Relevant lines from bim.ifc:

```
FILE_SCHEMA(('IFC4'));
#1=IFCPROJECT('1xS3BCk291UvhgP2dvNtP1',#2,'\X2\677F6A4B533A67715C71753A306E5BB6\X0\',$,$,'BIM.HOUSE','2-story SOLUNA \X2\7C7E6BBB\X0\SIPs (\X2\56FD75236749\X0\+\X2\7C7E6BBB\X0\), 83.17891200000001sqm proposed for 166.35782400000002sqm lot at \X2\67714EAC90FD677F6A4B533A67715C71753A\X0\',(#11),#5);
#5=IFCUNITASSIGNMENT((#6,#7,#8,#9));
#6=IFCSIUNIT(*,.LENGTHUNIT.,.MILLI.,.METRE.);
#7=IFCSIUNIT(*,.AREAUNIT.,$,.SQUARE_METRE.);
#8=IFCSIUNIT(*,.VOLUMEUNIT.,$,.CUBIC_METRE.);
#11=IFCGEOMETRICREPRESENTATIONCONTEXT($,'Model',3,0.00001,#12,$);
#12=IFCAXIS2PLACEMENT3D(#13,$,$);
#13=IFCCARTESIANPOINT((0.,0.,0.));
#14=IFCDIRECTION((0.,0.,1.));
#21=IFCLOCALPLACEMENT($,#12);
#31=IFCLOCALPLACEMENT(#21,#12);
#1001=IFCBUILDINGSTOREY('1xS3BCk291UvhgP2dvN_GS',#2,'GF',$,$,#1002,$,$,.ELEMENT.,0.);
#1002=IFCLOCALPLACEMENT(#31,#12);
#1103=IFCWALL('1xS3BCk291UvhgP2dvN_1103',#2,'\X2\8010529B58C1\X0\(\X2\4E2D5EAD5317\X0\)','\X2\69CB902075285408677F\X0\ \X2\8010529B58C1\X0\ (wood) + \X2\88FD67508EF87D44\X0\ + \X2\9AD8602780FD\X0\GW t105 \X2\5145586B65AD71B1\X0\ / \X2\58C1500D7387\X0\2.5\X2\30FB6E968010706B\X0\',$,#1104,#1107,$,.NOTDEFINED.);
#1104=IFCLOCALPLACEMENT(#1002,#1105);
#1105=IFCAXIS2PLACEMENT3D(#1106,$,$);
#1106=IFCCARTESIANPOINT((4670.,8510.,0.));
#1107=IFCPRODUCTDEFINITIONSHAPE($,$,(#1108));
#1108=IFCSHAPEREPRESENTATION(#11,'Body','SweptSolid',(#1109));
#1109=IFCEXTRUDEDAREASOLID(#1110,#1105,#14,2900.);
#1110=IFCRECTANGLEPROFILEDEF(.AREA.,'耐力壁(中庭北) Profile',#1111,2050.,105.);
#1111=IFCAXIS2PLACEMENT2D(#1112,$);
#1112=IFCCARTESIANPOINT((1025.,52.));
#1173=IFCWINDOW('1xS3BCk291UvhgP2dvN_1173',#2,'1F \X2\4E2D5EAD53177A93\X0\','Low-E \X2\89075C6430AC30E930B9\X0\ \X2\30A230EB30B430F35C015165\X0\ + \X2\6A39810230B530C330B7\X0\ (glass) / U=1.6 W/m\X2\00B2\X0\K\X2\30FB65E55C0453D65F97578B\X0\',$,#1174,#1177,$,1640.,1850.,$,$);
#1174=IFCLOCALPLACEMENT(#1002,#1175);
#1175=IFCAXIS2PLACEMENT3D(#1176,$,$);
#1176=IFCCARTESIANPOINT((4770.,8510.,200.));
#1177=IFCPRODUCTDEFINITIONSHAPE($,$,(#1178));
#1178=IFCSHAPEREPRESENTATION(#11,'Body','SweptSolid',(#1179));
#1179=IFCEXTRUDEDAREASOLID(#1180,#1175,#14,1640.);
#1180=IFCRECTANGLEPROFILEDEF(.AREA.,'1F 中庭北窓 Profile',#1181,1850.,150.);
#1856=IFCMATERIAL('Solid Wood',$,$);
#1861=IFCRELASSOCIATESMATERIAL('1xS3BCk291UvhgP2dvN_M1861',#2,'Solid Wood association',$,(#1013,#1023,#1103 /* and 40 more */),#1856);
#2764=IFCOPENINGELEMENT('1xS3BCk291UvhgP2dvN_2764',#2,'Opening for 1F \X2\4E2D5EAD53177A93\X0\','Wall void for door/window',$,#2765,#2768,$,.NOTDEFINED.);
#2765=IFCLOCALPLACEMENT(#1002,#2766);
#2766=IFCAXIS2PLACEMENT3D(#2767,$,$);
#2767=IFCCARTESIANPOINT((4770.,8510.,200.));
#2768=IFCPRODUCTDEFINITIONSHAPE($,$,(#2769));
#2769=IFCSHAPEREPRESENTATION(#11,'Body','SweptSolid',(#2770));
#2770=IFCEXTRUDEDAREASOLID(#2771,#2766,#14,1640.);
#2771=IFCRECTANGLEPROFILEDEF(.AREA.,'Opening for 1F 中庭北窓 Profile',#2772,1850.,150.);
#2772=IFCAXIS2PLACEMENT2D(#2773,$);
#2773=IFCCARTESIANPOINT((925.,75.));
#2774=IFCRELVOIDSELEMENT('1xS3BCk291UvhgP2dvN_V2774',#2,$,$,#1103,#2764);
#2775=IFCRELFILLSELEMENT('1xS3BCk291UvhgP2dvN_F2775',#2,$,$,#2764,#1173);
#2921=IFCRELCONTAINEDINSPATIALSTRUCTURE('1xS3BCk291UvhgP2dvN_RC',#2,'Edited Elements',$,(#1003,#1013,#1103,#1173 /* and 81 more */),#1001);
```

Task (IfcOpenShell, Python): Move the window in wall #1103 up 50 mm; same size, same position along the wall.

```python
import numpy as np
import ifcopenshell
import ifcopenshell.api.geometry
import ifcopenshell.util.placement
import ifcopenshell.util.unit

model = ifcopenshell.open("bim.ifc")
unit_scale = ifcopenshell.util.unit.calculate_unit_scale(model)

window = model.by_guid("1xS3BCk291UvhgP2dvN_1173")
opening = window.FillsVoids[0].RelatingOpeningElement
dz = 0.05 / unit_scale

shift = np.array([0.0, 0.0, dz])
# The window is not placed relative to its opening, so move both.
for product in (opening, window):
    matrix = ifcopenshell.util.placement.get_local_placement(product.ObjectPlacement)
    matrix[:3, 3] += shift
    ifcopenshell.api.geometry.edit_object_placement(model, product=product, matrix=matrix, is_si=False)

print(f"moved by {dz * unit_scale:+.3f} m")

model.write("bim_rev.ifc")
```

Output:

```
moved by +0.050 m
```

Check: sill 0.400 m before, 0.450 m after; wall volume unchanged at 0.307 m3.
